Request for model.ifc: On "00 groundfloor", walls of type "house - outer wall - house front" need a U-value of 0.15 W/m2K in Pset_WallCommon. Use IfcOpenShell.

First a look at what the model holds.

```python
import ifcopenshell
import ifcopenshell.util.element

model = ifcopenshell.open("model.ifc")
print(model.schema)
storey = next(s for s in model.by_type("IfcBuildingStorey") if s.Name == "00 groundfloor")
walls = [e for e in ifcopenshell.util.element.get_decomposition(storey) if e.is_a("IfcWall")]
seen = {}
for e in walls:
    element_type = ifcopenshell.util.element.get_type(e)
    key = (element_type.Name if element_type != e and element_type else None, ifcopenshell.util.element.get_pset(e, "Pset_WallCommon", "ThermalTransmittance"))
    seen[key] = seen.get(key, 0) + 1
for (name, value), count in sorted(seen.items(), key=str):
    print(count, "x", name, "|", value)
```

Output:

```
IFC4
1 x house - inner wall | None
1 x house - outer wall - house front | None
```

```python
import ifcopenshell
import ifcopenshell.api.pset
import ifcopenshell.util.element

model = ifcopenshell.open("model.ifc")

storey = next(s for s in model.by_type("IfcBuildingStorey") if s.Name == "00 groundfloor")
walls = [e for e in ifcopenshell.util.element.get_decomposition(storey) if e.is_a("IfcWall")]

count = 0
for e in walls:
    element_type = ifcopenshell.util.element.get_type(e)
    if element_type in (None, e) or element_type.Name != "house - outer wall - house front":
        continue
    # add_pset returns the element's existing set when there is one.
    pset = ifcopenshell.api.pset.add_pset(model, product=e, name="Pset_WallCommon")
    ifcopenshell.api.pset.edit_pset(model, pset=pset, properties={"ThermalTransmittance": 0.15})
    count += 1

print(count, "walls updated")

model.write("model-out.ifc")
```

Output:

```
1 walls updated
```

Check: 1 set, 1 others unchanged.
